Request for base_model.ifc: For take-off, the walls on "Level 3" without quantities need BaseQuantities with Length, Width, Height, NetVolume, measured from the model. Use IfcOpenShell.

First a look at what the model holds.

```python
import ifcopenshell
import ifcopenshell.util.element
import ifcopenshell.util.unit

model = ifcopenshell.open("base_model.ifc")
print(model.schema)
for unit_type in ("LENGTHUNIT", "AREAUNIT", "VOLUMEUNIT"):
    print(unit_type, ifcopenshell.util.unit.calculate_unit_scale(model, unit_type))
storey = next(s for s in model.by_type("IfcBuildingStorey") if s.Name == "Level 3")
walls = [e for e in ifcopenshell.util.element.get_decomposition(storey) if e.is_a("IfcWall")]
for e in sorted(walls, key=lambda e: e.id()):
    print(e.id(), e.is_a(), e.Name, list(ifcopenshell.util.element.get_psets(e, qtos_only=True)), sep=" | ")
```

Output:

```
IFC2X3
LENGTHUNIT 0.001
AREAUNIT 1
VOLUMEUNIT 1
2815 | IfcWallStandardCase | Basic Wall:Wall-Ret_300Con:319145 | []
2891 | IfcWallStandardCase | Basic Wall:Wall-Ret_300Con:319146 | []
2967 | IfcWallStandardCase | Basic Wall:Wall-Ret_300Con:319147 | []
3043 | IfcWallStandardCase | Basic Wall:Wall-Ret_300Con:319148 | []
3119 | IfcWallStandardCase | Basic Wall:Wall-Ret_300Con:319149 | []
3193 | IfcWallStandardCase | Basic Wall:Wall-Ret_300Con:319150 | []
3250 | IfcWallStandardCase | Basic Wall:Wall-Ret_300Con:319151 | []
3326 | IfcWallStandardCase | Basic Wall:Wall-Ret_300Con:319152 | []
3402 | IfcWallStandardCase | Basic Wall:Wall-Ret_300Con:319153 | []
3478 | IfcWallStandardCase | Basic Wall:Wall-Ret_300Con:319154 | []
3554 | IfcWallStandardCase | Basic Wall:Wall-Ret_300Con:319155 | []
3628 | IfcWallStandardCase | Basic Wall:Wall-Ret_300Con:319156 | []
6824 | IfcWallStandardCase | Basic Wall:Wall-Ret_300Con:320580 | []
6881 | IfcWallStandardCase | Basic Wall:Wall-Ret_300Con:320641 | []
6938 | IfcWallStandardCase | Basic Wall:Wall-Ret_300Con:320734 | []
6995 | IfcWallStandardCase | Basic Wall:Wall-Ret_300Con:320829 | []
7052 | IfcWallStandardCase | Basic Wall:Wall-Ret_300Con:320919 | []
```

```python
import ifcopenshell
import ifcopenshell.api.pset
import ifcopenshell.geom
import ifcopenshell.util.element
import ifcopenshell.util.shape
import ifcopenshell.util.unit

model = ifcopenshell.open("base_model.ifc")
unit_scale = ifcopenshell.util.unit.calculate_unit_scale(model)
volume_scale = ifcopenshell.util.unit.calculate_unit_scale(model, "VOLUMEUNIT")
settings = ifcopenshell.geom.settings()

storey = next(s for s in model.by_type("IfcBuildingStorey") if s.Name == "Level 3")
walls = [e for e in ifcopenshell.util.element.get_decomposition(storey) if e.is_a("IfcWall")]

for e in sorted(walls, key=lambda e: e.id()):
    if ifcopenshell.util.element.get_psets(e, qtos_only=True, should_inherit=False):
        continue
    # Geometry comes back in metres, in the element's own axes.
    shape = ifcopenshell.geom.create_shape(settings, e)
    values = {
        "Length": ifcopenshell.util.shape.get_x(shape.geometry) / unit_scale,
        "Width": ifcopenshell.util.shape.get_y(shape.geometry) / unit_scale,
        "Height": ifcopenshell.util.shape.get_z(shape.geometry) / unit_scale,
        "NetVolume": ifcopenshell.util.shape.get_volume(shape.geometry) / volume_scale,
    }
    qto = ifcopenshell.api.pset.add_qto(model, product=e, name="BaseQuantities")
    ifcopenshell.api.pset.edit_qto(model, qto=qto, properties=values)
    print(e.id(), {k: round(v, 3) for k, v in values.items()})

model.write("base_model_v2.ifc")
```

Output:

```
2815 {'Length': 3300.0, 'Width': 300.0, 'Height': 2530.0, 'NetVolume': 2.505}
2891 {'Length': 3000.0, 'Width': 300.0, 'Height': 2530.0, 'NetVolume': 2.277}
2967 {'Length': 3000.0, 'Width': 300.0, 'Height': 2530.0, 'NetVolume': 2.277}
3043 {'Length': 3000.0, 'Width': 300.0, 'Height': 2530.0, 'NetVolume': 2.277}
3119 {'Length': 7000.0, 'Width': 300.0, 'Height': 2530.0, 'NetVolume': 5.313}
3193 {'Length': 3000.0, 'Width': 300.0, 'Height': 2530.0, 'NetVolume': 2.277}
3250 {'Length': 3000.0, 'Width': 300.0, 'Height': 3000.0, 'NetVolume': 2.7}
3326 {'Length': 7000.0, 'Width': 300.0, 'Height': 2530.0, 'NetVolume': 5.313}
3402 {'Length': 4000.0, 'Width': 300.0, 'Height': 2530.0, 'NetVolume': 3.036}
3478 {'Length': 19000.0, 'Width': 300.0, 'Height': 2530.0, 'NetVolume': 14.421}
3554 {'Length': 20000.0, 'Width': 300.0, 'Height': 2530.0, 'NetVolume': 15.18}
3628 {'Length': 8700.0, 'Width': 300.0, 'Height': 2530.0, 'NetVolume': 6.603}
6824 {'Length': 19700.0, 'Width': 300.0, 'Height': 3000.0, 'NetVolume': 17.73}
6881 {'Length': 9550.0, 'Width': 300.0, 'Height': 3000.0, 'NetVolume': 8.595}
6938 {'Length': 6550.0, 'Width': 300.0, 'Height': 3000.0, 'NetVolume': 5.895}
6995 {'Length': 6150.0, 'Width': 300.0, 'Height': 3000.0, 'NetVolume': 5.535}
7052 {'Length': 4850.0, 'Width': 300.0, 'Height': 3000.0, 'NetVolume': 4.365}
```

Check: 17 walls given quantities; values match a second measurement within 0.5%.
